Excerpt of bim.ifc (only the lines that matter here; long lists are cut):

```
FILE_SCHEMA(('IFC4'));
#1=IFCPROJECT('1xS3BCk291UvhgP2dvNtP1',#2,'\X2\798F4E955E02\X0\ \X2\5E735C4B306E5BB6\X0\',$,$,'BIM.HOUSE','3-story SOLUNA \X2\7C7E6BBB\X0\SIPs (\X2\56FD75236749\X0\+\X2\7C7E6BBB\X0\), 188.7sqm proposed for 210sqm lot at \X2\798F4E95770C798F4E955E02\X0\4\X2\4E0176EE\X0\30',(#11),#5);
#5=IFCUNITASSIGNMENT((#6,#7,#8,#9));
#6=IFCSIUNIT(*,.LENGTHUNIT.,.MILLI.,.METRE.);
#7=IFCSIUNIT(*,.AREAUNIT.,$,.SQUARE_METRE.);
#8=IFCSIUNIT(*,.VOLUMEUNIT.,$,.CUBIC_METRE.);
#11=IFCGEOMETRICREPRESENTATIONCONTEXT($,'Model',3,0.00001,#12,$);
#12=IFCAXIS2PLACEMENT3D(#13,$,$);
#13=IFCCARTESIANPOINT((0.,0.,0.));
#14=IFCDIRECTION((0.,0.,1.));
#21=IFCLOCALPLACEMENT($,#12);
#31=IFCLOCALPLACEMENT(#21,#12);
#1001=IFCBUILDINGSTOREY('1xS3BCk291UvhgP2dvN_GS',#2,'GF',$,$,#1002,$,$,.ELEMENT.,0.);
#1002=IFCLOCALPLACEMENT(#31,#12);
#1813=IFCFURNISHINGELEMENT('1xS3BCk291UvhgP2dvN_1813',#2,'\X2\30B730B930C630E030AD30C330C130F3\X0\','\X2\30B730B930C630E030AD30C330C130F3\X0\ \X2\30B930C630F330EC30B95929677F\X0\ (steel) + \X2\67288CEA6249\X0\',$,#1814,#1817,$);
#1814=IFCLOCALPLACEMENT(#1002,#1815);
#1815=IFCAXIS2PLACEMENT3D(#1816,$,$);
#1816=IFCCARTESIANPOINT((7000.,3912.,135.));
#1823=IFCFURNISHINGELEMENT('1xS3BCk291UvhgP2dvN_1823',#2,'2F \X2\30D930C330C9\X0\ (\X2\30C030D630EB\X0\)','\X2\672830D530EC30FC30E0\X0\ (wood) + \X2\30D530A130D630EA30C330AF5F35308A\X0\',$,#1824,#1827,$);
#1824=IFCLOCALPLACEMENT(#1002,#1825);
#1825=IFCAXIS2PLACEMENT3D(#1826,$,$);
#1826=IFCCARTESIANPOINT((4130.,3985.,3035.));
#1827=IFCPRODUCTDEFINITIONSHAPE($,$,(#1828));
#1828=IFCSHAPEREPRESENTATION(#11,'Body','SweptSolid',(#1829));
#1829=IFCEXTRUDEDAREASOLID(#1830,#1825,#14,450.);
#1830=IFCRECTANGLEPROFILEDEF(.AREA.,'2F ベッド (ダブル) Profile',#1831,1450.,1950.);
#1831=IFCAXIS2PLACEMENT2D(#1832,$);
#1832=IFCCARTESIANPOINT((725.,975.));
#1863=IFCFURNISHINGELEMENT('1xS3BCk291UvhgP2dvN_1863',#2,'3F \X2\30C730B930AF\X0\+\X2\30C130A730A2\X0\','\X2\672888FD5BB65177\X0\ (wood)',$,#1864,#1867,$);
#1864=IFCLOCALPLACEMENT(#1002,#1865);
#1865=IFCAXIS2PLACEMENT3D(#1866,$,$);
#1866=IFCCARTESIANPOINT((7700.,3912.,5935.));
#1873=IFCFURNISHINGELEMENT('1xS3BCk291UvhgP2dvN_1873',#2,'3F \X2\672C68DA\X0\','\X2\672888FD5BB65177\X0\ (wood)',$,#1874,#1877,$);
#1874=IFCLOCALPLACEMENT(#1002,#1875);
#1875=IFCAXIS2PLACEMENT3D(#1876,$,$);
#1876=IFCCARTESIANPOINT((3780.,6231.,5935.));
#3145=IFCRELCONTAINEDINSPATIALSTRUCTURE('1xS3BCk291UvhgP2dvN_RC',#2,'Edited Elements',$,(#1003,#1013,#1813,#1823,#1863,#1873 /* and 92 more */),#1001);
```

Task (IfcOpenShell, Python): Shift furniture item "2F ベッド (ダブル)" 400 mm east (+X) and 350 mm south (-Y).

```python
import ifcopenshell
import ifcopenshell.api.geometry
import ifcopenshell.util.placement
import ifcopenshell.util.unit

model = ifcopenshell.open("bim.ifc")
unit_scale = ifcopenshell.util.unit.calculate_unit_scale(model)

item = model.by_id(1823)
matrix = ifcopenshell.util.placement.get_local_placement(item.ObjectPlacement)
matrix[0, 3] += 0.4 / unit_scale
matrix[1, 3] -= 0.35 / unit_scale
ifcopenshell.api.geometry.edit_object_placement(model, product=item, matrix=matrix, is_si=False)

print(ifcopenshell.util.placement.get_local_placement(item.ObjectPlacement).round(3) + 0.0)

model.write("bim_rev.ifc")
```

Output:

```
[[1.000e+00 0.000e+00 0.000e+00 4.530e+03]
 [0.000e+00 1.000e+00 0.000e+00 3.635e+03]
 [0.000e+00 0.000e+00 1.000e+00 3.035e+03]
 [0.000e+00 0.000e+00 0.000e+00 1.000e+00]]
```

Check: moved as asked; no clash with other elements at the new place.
